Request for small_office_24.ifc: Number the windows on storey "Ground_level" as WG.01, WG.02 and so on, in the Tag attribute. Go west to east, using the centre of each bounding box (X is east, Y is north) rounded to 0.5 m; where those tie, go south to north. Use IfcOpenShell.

First a look at what the model holds.

```python
import ifcopenshell
import ifcopenshell.util.element
import ifcopenshell.util.placement

model = ifcopenshell.open("small_office_24.ifc")
print(model.schema)
storey = next(s for s in model.by_type("IfcBuildingStorey") if s.Name == "Ground_level")
windows = [e for e in ifcopenshell.util.element.get_decomposition(storey) if e.is_a("IfcWindow")]
for e in sorted(windows, key=lambda e: e.id()):
    origin = ifcopenshell.util.placement.get_local_placement(e.ObjectPlacement)[:3, 3]
    print(e.id(), e.Tag, e.Name, origin.round(2) + 0.0, sep=" | ")
```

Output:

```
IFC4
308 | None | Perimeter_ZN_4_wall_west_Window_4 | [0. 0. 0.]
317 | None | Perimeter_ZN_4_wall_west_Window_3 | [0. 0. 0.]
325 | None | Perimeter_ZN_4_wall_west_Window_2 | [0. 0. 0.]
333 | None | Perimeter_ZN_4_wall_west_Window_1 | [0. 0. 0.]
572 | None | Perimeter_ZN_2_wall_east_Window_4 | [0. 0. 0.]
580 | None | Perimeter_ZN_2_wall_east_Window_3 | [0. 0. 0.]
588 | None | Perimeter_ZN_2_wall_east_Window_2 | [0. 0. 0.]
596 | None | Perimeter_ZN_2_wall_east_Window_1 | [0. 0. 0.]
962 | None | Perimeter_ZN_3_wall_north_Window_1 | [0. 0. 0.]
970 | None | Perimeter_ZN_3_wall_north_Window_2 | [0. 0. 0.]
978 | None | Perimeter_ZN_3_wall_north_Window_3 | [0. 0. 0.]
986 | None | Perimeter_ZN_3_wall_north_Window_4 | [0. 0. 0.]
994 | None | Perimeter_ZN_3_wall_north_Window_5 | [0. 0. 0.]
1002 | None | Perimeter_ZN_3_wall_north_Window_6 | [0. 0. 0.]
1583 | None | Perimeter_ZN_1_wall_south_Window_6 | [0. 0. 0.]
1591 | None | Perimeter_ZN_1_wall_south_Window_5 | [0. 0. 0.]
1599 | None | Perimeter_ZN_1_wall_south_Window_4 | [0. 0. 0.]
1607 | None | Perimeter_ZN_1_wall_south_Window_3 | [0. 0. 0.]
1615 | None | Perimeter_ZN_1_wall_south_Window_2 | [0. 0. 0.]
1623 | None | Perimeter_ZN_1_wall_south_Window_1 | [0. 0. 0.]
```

```python
import ifcopenshell
import ifcopenshell.geom
import ifcopenshell.util.element
import ifcopenshell.util.shape

model = ifcopenshell.open("small_office_24.ifc")
settings = ifcopenshell.geom.settings()
settings.set("use-world-coords", True)


def centre(element):
    shape = ifcopenshell.geom.create_shape(settings, element)
    return ifcopenshell.util.shape.get_bbox_centroid(shape.geometry)


storey = next(s for s in model.by_type("IfcBuildingStorey") if s.Name == "Ground_level")
windows = [e for e in ifcopenshell.util.element.get_decomposition(storey) if e.is_a("IfcWindow")]

# Insertion points can sit at a corner or the storey origin, so sort by the geometry (in metres).
centres = {e: centre(e) for e in windows}
windows.sort(key=lambda e: (round(centres[e][0] / 0.5), centres[e][1]))

for i, e in enumerate(windows, start=1):
    number = f"WG.{i:02d}"
    e.Tag = number
    print(e.id(), number)

model.write("small_office_24_v2.ifc")
```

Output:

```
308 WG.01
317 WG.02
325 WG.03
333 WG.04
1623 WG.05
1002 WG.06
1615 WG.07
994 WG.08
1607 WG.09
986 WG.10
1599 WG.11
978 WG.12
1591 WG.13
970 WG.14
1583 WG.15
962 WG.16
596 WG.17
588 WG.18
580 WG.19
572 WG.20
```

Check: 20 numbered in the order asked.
